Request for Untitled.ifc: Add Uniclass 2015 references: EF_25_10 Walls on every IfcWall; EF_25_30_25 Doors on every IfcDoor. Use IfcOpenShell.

First a look at what the model holds.

```python
import ifcopenshell

model = ifcopenshell.open("Untitled.ifc")
print(model.schema)
print("classifications:", [c.Name for c in model.by_type("IfcClassification")])
for ifc_class in ("IfcDoor", "IfcRoof", "IfcStair", "IfcWall", "IfcWindow"):
    print(ifc_class, len(model.by_type(ifc_class)))
```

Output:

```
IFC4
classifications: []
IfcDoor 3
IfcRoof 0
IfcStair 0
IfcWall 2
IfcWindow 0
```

```python
import ifcopenshell
import ifcopenshell.api.classification

model = ifcopenshell.open("Untitled.ifc")

system = ifcopenshell.api.classification.add_classification(model, classification="Uniclass 2015")

codes = {
    "IfcWall": ("EF_25_10", "Walls"),
    "IfcDoor": ("EF_25_30_25", "Doors"),
}
for ifc_class, (code, name) in codes.items():
    products = model.by_type(ifc_class)
    ifcopenshell.api.classification.add_reference(
        model, products=products, classification=system, identification=code, name=name
    )
    print(code, len(products))

model.write("Untitled_rev.ifc")
```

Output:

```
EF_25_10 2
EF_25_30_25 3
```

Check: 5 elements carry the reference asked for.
